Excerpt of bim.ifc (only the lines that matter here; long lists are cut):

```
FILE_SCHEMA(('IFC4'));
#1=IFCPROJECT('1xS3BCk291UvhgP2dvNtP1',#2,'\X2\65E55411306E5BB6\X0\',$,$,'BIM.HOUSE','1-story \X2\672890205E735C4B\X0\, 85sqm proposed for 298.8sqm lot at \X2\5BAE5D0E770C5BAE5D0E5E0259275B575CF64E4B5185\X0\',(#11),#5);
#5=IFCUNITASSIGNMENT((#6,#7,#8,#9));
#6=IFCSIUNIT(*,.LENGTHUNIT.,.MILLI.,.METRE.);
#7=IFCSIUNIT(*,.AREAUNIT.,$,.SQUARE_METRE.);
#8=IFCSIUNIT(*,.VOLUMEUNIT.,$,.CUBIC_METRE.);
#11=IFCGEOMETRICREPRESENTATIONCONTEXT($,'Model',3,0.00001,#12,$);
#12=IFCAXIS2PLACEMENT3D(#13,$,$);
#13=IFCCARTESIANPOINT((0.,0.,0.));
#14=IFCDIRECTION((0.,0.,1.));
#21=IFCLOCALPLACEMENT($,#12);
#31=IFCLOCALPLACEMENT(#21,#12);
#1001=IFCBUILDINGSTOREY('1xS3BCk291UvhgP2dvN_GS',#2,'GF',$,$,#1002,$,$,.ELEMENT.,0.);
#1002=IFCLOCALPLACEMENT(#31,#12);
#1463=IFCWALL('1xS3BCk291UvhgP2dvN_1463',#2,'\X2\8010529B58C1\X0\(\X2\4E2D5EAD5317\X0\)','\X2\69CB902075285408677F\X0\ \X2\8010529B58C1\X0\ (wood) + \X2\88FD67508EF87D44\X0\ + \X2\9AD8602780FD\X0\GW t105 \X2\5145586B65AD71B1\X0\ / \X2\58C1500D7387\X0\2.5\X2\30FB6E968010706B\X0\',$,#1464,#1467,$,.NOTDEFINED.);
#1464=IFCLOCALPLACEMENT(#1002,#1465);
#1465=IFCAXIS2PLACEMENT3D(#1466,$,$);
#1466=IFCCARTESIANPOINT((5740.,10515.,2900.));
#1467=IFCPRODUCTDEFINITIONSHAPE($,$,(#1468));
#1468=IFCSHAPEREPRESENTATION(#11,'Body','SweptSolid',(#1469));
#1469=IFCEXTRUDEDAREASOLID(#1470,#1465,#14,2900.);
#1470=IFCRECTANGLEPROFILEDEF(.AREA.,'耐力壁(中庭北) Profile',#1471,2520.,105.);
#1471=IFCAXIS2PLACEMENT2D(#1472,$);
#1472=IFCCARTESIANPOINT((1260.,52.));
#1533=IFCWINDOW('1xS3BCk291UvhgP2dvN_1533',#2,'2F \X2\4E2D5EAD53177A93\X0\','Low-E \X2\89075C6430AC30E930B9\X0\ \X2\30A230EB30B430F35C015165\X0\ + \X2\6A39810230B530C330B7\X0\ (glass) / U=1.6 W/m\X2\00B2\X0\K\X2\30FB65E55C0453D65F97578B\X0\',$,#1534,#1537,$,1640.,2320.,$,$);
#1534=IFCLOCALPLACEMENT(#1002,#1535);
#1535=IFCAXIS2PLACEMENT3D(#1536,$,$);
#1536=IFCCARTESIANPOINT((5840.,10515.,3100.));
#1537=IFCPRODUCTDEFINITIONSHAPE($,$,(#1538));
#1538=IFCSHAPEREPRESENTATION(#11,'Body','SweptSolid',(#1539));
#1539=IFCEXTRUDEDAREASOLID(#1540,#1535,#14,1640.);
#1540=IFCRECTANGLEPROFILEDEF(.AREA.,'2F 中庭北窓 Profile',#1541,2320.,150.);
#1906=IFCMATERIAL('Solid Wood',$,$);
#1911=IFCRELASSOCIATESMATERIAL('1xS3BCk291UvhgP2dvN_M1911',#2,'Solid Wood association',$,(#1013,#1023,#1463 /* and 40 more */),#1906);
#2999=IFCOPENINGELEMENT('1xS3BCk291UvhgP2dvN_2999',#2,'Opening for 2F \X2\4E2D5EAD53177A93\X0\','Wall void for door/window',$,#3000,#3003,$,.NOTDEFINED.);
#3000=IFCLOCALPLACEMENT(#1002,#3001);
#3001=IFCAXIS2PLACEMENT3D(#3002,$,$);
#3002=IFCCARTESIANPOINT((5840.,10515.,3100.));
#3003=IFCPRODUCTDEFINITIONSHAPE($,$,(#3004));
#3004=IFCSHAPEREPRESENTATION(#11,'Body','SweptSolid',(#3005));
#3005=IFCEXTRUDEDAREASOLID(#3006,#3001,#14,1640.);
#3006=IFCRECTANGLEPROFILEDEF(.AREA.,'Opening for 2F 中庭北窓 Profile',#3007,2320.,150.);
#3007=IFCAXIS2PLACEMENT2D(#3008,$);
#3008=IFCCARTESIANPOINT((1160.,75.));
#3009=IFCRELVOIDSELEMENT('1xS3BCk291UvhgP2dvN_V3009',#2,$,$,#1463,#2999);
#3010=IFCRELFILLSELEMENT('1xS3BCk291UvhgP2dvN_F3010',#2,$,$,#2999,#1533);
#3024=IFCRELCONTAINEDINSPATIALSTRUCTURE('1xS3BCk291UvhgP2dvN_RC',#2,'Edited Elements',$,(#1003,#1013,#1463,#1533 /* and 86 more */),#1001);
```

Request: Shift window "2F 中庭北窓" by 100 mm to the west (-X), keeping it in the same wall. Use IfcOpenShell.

```python
import ifcopenshell
import ifcopenshell.api.geometry
import ifcopenshell.util.placement
import ifcopenshell.util.unit

model = ifcopenshell.open("bim.ifc")
unit_scale = ifcopenshell.util.unit.calculate_unit_scale(model)

window = model.by_guid("1xS3BCk291UvhgP2dvN_1533")
opening = window.FillsVoids[0].RelatingOpeningElement
wall = opening.VoidsElements[0].RelatingBuildingElement

wall_matrix = ifcopenshell.util.placement.get_local_placement(wall.ObjectPlacement)
shift = wall_matrix[:3, 0] * -0.1 / unit_scale
before = ifcopenshell.util.placement.get_local_placement(window.ObjectPlacement)[:3, 3].copy()

# The window is not placed relative to its opening, so move both.
for product in (opening, window):
    matrix = ifcopenshell.util.placement.get_local_placement(product.ObjectPlacement)
    matrix[:3, 3] += shift
    ifcopenshell.api.geometry.edit_object_placement(model, product=product, matrix=matrix, is_si=False)

after = ifcopenshell.util.placement.get_local_placement(window.ObjectPlacement)[:3, 3]
print("window moved by", (after - before).round(3) + 0.0)

model.write("bim_updated.ifc")
```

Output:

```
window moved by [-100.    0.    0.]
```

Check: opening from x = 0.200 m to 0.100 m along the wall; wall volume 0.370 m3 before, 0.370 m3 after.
